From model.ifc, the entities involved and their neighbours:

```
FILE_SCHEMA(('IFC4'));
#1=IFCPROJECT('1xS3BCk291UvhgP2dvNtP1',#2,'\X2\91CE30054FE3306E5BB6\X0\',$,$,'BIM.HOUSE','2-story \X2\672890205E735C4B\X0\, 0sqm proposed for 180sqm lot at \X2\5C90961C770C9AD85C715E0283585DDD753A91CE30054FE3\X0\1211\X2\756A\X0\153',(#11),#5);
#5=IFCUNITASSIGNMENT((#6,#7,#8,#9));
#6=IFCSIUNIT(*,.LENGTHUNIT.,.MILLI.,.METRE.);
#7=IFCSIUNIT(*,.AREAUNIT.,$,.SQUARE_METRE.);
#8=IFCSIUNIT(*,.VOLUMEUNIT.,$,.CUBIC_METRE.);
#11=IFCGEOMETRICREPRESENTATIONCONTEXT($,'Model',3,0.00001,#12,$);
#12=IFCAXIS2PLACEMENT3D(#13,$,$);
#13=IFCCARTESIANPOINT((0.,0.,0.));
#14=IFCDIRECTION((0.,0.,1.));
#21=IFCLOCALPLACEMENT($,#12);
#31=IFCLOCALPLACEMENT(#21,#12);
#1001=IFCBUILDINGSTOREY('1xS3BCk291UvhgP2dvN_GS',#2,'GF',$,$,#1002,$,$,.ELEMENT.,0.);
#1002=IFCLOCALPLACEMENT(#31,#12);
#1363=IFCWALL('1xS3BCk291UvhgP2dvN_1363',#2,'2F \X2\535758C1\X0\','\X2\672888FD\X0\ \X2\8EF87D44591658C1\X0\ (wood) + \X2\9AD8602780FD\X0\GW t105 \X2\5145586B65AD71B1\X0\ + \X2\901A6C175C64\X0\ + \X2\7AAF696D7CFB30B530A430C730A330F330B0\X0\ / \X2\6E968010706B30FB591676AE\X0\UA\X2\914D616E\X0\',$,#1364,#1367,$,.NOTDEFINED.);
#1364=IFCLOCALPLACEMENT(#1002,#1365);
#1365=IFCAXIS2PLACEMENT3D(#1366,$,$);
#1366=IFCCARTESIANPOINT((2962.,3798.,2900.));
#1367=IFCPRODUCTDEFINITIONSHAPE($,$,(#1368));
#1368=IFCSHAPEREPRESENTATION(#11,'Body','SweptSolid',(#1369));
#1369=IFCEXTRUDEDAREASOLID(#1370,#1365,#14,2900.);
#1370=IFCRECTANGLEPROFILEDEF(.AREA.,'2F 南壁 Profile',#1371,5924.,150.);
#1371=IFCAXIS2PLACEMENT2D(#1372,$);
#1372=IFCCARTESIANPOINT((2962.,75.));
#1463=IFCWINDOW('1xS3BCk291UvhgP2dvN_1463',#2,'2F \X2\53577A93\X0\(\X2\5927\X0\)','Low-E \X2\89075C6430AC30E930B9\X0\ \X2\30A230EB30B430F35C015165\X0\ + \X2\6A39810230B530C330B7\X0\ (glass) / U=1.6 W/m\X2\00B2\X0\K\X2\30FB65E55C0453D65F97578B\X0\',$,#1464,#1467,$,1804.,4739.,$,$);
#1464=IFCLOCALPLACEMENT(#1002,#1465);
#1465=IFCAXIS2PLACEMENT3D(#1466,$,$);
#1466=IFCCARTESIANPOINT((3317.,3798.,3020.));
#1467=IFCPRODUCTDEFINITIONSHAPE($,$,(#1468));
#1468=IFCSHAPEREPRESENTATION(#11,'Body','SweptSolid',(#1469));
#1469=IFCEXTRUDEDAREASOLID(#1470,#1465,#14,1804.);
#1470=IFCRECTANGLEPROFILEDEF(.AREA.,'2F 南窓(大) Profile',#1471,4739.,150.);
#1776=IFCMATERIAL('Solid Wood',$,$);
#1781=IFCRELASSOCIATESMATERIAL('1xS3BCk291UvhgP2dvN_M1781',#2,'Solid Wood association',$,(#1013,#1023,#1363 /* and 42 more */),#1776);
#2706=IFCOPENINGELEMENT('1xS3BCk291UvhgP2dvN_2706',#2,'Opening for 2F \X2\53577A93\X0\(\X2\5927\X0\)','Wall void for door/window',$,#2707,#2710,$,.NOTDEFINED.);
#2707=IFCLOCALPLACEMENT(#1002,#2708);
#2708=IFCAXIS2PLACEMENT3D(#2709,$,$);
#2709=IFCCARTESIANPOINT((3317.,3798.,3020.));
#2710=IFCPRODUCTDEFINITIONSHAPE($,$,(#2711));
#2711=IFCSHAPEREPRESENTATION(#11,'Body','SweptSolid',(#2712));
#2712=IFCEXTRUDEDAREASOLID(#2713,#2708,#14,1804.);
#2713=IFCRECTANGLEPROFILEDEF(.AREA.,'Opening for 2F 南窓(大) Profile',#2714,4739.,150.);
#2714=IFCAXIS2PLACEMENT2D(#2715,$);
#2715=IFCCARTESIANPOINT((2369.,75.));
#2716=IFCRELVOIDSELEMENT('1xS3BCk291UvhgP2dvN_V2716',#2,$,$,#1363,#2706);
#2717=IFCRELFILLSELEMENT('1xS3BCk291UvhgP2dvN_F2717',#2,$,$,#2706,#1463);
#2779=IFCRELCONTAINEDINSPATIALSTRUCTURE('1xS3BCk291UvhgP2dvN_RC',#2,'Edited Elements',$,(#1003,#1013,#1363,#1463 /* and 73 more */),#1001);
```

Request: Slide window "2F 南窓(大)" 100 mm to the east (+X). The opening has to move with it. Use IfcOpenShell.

```python
import ifcopenshell
import ifcopenshell.api.geometry
import ifcopenshell.util.placement
import ifcopenshell.util.unit

model = ifcopenshell.open("model.ifc")
unit_scale = ifcopenshell.util.unit.calculate_unit_scale(model)

window = model.by_id(1463)
opening = window.FillsVoids[0].RelatingOpeningElement
wall = opening.VoidsElements[0].RelatingBuildingElement

wall_matrix = ifcopenshell.util.placement.get_local_placement(wall.ObjectPlacement)
shift = wall_matrix[:3, 0] * 0.1 / unit_scale
before = ifcopenshell.util.placement.get_local_placement(window.ObjectPlacement)[:3, 3].copy()

# The window is not placed relative to its opening, so move both.
for product in (opening, window):
    matrix = ifcopenshell.util.placement.get_local_placement(product.ObjectPlacement)
    matrix[:3, 3] += shift
    ifcopenshell.api.geometry.edit_object_placement(model, product=product, matrix=matrix, is_si=False)

after = ifcopenshell.util.placement.get_local_placement(window.ObjectPlacement)[:3, 3]
print("window moved by", (after - before).round(3) + 0.0)

model.write("model_updated.ifc")
```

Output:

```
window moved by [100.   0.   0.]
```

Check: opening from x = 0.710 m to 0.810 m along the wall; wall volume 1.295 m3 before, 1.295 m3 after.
